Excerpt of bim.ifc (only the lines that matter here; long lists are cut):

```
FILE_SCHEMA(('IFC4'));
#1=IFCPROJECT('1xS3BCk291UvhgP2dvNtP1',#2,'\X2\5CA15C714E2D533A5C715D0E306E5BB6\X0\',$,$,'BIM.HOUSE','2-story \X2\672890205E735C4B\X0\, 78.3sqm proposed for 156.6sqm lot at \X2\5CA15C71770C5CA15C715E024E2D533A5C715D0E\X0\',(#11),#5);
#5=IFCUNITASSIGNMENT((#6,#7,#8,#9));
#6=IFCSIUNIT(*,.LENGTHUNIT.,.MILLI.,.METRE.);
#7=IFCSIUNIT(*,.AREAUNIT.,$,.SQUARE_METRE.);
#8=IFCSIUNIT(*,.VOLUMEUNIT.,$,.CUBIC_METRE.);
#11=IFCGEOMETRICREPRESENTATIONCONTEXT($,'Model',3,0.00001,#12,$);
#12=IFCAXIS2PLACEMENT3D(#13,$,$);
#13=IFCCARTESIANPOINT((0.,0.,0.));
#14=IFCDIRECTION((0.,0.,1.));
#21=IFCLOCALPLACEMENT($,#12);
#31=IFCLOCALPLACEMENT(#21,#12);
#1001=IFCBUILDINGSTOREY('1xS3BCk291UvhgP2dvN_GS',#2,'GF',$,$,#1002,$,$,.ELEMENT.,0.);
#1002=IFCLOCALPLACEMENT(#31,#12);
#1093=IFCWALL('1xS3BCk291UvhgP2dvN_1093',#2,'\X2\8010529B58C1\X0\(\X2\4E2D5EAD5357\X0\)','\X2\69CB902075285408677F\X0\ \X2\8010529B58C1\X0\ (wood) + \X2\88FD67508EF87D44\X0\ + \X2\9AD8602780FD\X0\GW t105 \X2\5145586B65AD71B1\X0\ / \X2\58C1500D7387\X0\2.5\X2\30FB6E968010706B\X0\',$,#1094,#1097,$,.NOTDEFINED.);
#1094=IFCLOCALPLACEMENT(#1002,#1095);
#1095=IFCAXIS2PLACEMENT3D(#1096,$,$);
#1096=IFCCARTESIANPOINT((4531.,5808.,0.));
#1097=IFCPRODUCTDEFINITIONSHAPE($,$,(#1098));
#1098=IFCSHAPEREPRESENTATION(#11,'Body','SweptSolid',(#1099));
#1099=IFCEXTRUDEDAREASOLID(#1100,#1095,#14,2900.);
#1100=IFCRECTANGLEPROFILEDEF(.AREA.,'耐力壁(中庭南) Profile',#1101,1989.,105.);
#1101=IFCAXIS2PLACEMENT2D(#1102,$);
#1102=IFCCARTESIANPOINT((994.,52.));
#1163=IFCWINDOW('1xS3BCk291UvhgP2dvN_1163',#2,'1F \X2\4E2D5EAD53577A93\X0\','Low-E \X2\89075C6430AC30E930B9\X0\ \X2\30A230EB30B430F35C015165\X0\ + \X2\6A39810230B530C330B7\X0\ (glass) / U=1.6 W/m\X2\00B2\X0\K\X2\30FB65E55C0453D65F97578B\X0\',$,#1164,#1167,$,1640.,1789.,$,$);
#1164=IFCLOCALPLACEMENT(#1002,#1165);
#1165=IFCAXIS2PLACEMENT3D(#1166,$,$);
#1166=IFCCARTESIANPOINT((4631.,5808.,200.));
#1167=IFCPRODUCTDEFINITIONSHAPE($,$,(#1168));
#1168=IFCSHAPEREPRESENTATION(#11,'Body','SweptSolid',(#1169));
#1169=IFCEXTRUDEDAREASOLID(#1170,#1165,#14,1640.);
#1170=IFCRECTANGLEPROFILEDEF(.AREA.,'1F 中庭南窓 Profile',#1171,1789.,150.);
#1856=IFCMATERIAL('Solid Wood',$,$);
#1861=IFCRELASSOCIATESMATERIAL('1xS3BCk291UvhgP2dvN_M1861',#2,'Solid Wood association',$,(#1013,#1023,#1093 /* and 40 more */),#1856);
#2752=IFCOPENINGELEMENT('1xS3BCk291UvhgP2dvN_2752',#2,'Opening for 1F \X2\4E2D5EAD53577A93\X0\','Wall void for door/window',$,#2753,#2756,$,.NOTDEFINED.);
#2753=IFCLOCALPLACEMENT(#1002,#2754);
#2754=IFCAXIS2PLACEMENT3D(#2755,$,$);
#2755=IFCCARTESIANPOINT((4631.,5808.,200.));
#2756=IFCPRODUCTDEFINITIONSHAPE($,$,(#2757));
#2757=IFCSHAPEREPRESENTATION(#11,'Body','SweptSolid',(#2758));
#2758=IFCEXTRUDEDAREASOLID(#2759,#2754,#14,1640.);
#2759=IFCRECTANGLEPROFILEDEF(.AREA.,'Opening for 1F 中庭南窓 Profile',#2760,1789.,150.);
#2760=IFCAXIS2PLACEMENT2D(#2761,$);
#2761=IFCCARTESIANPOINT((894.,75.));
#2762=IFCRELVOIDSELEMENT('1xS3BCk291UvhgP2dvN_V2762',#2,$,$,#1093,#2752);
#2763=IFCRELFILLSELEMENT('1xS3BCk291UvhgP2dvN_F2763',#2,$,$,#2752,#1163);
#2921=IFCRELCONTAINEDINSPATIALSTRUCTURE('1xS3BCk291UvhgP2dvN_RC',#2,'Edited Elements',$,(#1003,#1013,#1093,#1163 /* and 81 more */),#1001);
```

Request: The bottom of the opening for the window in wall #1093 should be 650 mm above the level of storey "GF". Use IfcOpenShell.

```python
import numpy as np
import ifcopenshell
import ifcopenshell.api.geometry
import ifcopenshell.geom
import ifcopenshell.util.element
import ifcopenshell.util.placement
import ifcopenshell.util.shape
import ifcopenshell.util.unit

model = ifcopenshell.open("bim.ifc")
unit_scale = ifcopenshell.util.unit.calculate_unit_scale(model)

window = model.by_guid("1xS3BCk291UvhgP2dvN_1163")
opening = window.FillsVoids[0].RelatingOpeningElement
storey = ifcopenshell.util.element.get_container(window, ifc_class="IfcBuildingStorey")
level = ifcopenshell.util.placement.get_local_placement(storey.ObjectPlacement)[2, 3]

# The opening's origin need not be at the sill, so measure its lowest point.
shape = ifcopenshell.geom.create_shape(ifcopenshell.geom.settings(), opening)
bottom = ifcopenshell.util.shape.get_shape_bottom_elevation(shape, shape.geometry) / unit_scale
dz = level + 0.65 / unit_scale - bottom

shift = np.array([0.0, 0.0, dz])
# The window is not placed relative to its opening, so move both.
for product in (opening, window):
    matrix = ifcopenshell.util.placement.get_local_placement(product.ObjectPlacement)
    matrix[:3, 3] += shift
    ifcopenshell.api.geometry.edit_object_placement(model, product=product, matrix=matrix, is_si=False)

print(f"moved by {dz * unit_scale:+.3f} m")

model.write("bim_rev.ifc")
```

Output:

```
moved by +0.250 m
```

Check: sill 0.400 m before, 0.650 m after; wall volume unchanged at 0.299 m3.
